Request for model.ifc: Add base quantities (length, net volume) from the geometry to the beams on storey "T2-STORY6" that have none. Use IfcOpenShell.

First a look at what the model holds.

```python
import ifcopenshell
import ifcopenshell.util.element
import ifcopenshell.util.unit

model = ifcopenshell.open("model.ifc")
print(model.schema)
for unit_type in ("LENGTHUNIT", "AREAUNIT", "VOLUMEUNIT"):
    print(unit_type, ifcopenshell.util.unit.calculate_unit_scale(model, unit_type))
storey = next(s for s in model.by_type("IfcBuildingStorey") if s.Name == "T2-STORY6")
beams = [e for e in ifcopenshell.util.element.get_decomposition(storey) if e.is_a("IfcBeam")]
for e in sorted(beams, key=lambda e: e.id()):
    print(e.id(), e.is_a(), e.Name, list(ifcopenshell.util.element.get_psets(e, qtos_only=True)), sep=" | ")
```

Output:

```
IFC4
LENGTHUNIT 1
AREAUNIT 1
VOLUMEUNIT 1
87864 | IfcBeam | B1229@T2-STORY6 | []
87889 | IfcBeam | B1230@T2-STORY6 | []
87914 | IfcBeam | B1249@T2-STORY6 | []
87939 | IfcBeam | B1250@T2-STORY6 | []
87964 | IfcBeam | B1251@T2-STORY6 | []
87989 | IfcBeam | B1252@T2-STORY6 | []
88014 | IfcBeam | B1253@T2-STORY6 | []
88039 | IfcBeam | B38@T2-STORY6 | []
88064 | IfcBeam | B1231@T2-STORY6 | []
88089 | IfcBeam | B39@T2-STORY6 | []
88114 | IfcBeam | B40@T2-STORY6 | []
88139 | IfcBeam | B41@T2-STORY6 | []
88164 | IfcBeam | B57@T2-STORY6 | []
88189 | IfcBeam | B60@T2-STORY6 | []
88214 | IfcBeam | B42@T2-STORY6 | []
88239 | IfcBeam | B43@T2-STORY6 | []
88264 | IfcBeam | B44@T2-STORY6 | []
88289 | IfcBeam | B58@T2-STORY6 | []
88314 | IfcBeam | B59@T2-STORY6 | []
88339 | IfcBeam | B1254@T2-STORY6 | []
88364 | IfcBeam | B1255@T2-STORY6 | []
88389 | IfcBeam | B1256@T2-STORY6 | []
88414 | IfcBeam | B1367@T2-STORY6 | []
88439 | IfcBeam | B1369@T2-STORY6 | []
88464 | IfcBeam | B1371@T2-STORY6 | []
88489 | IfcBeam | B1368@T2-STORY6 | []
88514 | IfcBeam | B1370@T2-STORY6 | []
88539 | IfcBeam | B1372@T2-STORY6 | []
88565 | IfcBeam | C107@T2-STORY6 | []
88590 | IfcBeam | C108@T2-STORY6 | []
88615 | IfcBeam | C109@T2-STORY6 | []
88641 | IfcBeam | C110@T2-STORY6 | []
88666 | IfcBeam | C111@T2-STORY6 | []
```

```python
import ifcopenshell
import ifcopenshell.api.pset
import ifcopenshell.geom
import ifcopenshell.util.element
import ifcopenshell.util.shape
import ifcopenshell.util.unit

model = ifcopenshell.open("model.ifc")
unit_scale = ifcopenshell.util.unit.calculate_unit_scale(model)
volume_scale = ifcopenshell.util.unit.calculate_unit_scale(model, "VOLUMEUNIT")
settings = ifcopenshell.geom.settings()

storey = next(s for s in model.by_type("IfcBuildingStorey") if s.Name == "T2-STORY6")
beams = [e for e in ifcopenshell.util.element.get_decomposition(storey) if e.is_a("IfcBeam")]

for e in sorted(beams, key=lambda e: e.id()):
    if ifcopenshell.util.element.get_psets(e, qtos_only=True, should_inherit=False):
        continue
    # Geometry comes back in metres, in the element's own axes.
    shape = ifcopenshell.geom.create_shape(settings, e)
    values = {
        "Length": ifcopenshell.util.shape.get_max_xyz(shape.geometry) / unit_scale,
        "NetVolume": ifcopenshell.util.shape.get_volume(shape.geometry) / volume_scale,
    }
    qto = ifcopenshell.api.pset.add_qto(model, product=e, name="Qto_BeamBaseQuantities")
    ifcopenshell.api.pset.edit_qto(model, qto=qto, properties=values)
    print(e.id(), {k: round(v, 3) for k, v in values.items()})

model.write("model_rev.ifc")
```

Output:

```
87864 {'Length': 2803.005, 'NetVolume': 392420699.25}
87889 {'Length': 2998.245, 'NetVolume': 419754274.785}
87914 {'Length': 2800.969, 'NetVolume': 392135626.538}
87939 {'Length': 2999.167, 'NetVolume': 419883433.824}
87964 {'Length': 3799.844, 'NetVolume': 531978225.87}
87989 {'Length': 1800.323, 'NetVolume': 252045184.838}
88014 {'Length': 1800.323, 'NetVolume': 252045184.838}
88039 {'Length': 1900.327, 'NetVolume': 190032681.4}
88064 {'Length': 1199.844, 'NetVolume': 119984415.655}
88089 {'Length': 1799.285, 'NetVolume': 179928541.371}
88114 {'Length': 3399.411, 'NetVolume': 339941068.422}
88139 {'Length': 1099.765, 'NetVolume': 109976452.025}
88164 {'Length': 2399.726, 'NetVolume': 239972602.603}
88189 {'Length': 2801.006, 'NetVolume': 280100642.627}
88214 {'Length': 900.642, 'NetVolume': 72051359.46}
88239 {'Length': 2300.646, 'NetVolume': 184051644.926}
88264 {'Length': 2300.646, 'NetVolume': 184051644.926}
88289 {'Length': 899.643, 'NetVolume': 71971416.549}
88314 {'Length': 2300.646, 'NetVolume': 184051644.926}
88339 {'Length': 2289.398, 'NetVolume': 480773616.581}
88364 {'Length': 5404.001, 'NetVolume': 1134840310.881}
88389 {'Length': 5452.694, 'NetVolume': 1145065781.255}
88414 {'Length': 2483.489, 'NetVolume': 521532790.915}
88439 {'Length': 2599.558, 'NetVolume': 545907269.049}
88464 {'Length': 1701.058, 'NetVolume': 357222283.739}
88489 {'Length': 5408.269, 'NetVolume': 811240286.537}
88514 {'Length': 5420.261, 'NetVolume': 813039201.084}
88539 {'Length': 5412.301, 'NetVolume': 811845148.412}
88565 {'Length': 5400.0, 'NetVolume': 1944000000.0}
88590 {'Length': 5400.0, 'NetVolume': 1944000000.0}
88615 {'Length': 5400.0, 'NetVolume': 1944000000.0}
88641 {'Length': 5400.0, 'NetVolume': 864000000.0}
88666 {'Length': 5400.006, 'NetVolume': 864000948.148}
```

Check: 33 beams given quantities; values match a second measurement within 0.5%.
